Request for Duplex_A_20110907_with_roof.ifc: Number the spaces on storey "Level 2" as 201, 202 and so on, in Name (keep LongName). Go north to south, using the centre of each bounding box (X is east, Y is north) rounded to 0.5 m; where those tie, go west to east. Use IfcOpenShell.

First a look at what the model holds.

```python
import ifcopenshell
import ifcopenshell.util.element
import ifcopenshell.util.placement

model = ifcopenshell.open("Duplex_A_20110907_with_roof.ifc")
print(model.schema)
storey = next(s for s in model.by_type("IfcBuildingStorey") if s.Name == "Level 2")
spaces = [e for e in ifcopenshell.util.element.get_decomposition(storey) if e.is_a("IfcSpace")]
for e in sorted(spaces, key=lambda e: e.id()):
    origin = ifcopenshell.util.placement.get_local_placement(e.ObjectPlacement)[:3, 3]
    print(e.id(), e.Name, e.LongName, origin.round(2) + 0.0, sep=" | ")
```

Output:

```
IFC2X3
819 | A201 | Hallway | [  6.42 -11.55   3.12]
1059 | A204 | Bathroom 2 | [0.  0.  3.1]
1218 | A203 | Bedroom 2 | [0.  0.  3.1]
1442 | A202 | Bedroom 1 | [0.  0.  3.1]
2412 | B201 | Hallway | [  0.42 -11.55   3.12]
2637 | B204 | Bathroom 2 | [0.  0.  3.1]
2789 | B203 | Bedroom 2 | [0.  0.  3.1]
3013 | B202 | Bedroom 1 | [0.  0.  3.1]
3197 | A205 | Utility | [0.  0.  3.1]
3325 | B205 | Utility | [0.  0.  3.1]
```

```python
import ifcopenshell
import ifcopenshell.geom
import ifcopenshell.util.element
import ifcopenshell.util.shape

model = ifcopenshell.open("Duplex_A_20110907_with_roof.ifc")
settings = ifcopenshell.geom.settings()
settings.set("use-world-coords", True)


def centre(element):
    shape = ifcopenshell.geom.create_shape(settings, element)
    return ifcopenshell.util.shape.get_bbox_centroid(shape.geometry)


storey = next(s for s in model.by_type("IfcBuildingStorey") if s.Name == "Level 2")
spaces = [e for e in ifcopenshell.util.element.get_decomposition(storey) if e.is_a("IfcSpace")]

# Insertion points can sit at a corner or the storey origin, so sort by the geometry (in metres).
centres = {e: centre(e) for e in spaces}
spaces.sort(key=lambda e: (-round(centres[e][1] / 0.5), centres[e][0]))

for i, e in enumerate(spaces, start=1):
    number = f"2{i:02d}"
    e.Name = number
    print(e.id(), number)

model.write("Duplex_A_20110907_with_roof_updated.ifc")
```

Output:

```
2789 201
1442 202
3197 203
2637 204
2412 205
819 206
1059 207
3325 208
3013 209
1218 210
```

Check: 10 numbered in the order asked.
